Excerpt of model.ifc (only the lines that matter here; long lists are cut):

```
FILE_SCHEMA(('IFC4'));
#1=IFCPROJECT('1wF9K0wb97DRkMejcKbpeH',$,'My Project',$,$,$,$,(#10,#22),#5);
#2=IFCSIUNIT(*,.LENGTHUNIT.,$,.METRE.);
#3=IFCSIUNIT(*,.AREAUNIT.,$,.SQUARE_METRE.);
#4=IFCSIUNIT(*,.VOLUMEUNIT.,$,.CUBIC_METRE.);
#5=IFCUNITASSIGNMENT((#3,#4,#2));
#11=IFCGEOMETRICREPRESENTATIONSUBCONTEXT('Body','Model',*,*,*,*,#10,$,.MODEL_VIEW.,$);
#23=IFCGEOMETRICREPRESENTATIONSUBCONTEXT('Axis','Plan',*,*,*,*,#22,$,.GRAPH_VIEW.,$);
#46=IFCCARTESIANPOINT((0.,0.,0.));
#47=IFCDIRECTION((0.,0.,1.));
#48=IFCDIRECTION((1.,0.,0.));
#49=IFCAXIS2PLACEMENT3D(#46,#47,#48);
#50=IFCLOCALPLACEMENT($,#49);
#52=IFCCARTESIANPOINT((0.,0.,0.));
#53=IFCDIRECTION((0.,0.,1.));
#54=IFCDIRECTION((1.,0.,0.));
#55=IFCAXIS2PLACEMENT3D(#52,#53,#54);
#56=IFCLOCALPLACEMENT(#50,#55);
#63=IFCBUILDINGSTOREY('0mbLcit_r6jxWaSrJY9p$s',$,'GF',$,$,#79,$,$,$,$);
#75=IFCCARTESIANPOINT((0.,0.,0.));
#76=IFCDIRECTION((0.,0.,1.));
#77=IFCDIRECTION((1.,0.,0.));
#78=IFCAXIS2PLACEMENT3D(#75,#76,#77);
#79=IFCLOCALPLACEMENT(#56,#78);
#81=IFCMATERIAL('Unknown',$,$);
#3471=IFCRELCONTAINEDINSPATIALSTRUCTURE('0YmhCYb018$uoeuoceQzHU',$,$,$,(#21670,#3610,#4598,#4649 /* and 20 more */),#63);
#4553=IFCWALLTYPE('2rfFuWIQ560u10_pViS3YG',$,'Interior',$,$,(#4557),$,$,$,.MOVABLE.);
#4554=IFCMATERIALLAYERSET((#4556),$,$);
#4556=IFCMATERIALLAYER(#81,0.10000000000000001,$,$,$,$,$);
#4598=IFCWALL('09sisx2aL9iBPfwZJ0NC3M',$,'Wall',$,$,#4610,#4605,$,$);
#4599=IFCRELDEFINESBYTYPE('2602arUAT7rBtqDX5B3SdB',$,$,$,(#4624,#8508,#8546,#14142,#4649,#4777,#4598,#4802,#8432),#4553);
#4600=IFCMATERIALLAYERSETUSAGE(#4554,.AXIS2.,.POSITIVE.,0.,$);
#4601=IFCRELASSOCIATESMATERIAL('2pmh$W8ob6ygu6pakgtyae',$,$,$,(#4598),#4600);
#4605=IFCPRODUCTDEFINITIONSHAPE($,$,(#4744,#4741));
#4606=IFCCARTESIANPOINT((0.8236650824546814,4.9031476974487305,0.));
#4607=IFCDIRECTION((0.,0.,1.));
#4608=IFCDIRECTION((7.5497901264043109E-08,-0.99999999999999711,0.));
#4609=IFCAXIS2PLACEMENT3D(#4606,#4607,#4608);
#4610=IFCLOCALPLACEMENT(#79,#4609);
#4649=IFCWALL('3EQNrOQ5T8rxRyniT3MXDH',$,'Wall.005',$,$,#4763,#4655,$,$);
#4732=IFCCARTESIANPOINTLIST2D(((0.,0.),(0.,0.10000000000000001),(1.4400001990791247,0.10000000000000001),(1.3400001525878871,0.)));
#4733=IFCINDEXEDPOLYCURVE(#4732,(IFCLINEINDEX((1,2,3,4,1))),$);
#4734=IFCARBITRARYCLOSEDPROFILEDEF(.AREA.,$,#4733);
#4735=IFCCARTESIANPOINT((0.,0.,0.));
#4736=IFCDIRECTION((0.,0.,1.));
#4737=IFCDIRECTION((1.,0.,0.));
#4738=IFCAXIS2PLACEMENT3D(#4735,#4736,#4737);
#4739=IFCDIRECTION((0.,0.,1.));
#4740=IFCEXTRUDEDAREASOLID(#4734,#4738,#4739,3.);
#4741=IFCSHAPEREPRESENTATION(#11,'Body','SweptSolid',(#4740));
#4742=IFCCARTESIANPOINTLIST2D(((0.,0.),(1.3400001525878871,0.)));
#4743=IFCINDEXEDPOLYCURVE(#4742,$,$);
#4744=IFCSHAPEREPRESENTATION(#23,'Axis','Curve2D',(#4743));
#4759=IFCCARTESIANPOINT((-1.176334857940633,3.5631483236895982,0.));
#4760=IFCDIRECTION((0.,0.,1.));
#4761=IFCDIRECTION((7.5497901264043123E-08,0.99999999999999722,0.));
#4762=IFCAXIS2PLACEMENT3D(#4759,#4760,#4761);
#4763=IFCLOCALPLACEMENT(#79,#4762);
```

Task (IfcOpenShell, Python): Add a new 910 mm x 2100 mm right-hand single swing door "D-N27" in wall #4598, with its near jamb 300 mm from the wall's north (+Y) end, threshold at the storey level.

```python
import numpy as np
import ifcopenshell
import ifcopenshell.api.feature
import ifcopenshell.api.geometry
import ifcopenshell.api.root
import ifcopenshell.api.spatial
import ifcopenshell.geom
import ifcopenshell.util.element
import ifcopenshell.util.placement
import ifcopenshell.util.representation
import ifcopenshell.util.shape
import ifcopenshell.util.unit

model = ifcopenshell.open("model.ifc")
unit_scale = ifcopenshell.util.unit.calculate_unit_scale(model)
settings = ifcopenshell.geom.settings()


def volume(element):
    """Net volume in cubic metres, openings subtracted."""
    shape = ifcopenshell.geom.create_shape(settings, element)
    return ifcopenshell.util.shape.get_volume(shape.geometry)


wall = model.by_id(4598)
storey = ifcopenshell.util.element.get_container(wall, ifc_class="IfcBuildingStorey")
context = ifcopenshell.util.representation.get_context(model, "Model", "Body", "MODEL_VIEW")
before = volume(wall)

width, height, from_end, sill = 0.91, 2.1, 0.3, 0.0  # metres

# The wall runs along its own X axis, and the end named is its -X end.
wall_shape = ifcopenshell.geom.create_shape(settings, wall)
x, y, z = ifcopenshell.util.shape.get_vertices(wall_shape.geometry).T
start = x.min() + from_end
face, thickness = float(y.min()), float(y.max() - y.min())
wall_matrix = ifcopenshell.util.placement.get_local_placement(wall.ObjectPlacement)
level = ifcopenshell.util.placement.get_local_placement(storey.ObjectPlacement)[2, 3]


def in_wall(x, y):
    """Placement at x, y metres in the wall's axes, at sill height."""
    matrix = wall_matrix.copy()
    matrix[:, 3] = wall_matrix @ np.array([x / unit_scale, y / unit_scale, 0.0, 1.0])
    matrix[2, 3] = level + sill / unit_scale
    return matrix


# Opening: a box that overshoots both wall faces by 50 mm.
opening = ifcopenshell.api.root.create_entity(model, ifc_class="IfcOpeningElement", predefined_type="OPENING")
box = ifcopenshell.api.geometry.add_wall_representation(
    model, context=context, length=width, height=height, thickness=thickness + 0.1
)
ifcopenshell.api.geometry.assign_representation(model, product=opening, representation=box)
ifcopenshell.api.geometry.edit_object_placement(model, product=opening, matrix=in_wall(start, face - 0.05), is_si=False)
ifcopenshell.api.feature.add_feature(model, feature=opening, element=wall)

door = ifcopenshell.api.root.create_entity(model, ifc_class="IfcDoor", name="D-N27", predefined_type="DOOR")
door.OverallWidth, door.OverallHeight = width / unit_scale, height / unit_scale
door.OperationType = "SINGLE_SWING_RIGHT"
body = ifcopenshell.api.geometry.add_door_representation(
    model,
    context=context,
    overall_width=door.OverallWidth,
    overall_height=door.OverallHeight,
    operation_type="SINGLE_SWING_RIGHT",
    lining_properties={"LiningDepth": thickness / unit_scale, "ThresholdDepth": thickness / unit_scale},
)
ifcopenshell.api.geometry.assign_representation(model, product=door, representation=body)
ifcopenshell.api.spatial.assign_container(model, products=[door], relating_structure=storey)
ifcopenshell.api.feature.add_filling(model, opening=opening, element=door)

# The lining spans the wall, so the door starts at the wall face.
ifcopenshell.api.geometry.edit_object_placement(model, product=door, matrix=in_wall(start, face), is_si=False)

after = volume(wall)

print(f"wall volume {before:.3f} -> {after:.3f} m3")

model.write("model_rev.ifc")
```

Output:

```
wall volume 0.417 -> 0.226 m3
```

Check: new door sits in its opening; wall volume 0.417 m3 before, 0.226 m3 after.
